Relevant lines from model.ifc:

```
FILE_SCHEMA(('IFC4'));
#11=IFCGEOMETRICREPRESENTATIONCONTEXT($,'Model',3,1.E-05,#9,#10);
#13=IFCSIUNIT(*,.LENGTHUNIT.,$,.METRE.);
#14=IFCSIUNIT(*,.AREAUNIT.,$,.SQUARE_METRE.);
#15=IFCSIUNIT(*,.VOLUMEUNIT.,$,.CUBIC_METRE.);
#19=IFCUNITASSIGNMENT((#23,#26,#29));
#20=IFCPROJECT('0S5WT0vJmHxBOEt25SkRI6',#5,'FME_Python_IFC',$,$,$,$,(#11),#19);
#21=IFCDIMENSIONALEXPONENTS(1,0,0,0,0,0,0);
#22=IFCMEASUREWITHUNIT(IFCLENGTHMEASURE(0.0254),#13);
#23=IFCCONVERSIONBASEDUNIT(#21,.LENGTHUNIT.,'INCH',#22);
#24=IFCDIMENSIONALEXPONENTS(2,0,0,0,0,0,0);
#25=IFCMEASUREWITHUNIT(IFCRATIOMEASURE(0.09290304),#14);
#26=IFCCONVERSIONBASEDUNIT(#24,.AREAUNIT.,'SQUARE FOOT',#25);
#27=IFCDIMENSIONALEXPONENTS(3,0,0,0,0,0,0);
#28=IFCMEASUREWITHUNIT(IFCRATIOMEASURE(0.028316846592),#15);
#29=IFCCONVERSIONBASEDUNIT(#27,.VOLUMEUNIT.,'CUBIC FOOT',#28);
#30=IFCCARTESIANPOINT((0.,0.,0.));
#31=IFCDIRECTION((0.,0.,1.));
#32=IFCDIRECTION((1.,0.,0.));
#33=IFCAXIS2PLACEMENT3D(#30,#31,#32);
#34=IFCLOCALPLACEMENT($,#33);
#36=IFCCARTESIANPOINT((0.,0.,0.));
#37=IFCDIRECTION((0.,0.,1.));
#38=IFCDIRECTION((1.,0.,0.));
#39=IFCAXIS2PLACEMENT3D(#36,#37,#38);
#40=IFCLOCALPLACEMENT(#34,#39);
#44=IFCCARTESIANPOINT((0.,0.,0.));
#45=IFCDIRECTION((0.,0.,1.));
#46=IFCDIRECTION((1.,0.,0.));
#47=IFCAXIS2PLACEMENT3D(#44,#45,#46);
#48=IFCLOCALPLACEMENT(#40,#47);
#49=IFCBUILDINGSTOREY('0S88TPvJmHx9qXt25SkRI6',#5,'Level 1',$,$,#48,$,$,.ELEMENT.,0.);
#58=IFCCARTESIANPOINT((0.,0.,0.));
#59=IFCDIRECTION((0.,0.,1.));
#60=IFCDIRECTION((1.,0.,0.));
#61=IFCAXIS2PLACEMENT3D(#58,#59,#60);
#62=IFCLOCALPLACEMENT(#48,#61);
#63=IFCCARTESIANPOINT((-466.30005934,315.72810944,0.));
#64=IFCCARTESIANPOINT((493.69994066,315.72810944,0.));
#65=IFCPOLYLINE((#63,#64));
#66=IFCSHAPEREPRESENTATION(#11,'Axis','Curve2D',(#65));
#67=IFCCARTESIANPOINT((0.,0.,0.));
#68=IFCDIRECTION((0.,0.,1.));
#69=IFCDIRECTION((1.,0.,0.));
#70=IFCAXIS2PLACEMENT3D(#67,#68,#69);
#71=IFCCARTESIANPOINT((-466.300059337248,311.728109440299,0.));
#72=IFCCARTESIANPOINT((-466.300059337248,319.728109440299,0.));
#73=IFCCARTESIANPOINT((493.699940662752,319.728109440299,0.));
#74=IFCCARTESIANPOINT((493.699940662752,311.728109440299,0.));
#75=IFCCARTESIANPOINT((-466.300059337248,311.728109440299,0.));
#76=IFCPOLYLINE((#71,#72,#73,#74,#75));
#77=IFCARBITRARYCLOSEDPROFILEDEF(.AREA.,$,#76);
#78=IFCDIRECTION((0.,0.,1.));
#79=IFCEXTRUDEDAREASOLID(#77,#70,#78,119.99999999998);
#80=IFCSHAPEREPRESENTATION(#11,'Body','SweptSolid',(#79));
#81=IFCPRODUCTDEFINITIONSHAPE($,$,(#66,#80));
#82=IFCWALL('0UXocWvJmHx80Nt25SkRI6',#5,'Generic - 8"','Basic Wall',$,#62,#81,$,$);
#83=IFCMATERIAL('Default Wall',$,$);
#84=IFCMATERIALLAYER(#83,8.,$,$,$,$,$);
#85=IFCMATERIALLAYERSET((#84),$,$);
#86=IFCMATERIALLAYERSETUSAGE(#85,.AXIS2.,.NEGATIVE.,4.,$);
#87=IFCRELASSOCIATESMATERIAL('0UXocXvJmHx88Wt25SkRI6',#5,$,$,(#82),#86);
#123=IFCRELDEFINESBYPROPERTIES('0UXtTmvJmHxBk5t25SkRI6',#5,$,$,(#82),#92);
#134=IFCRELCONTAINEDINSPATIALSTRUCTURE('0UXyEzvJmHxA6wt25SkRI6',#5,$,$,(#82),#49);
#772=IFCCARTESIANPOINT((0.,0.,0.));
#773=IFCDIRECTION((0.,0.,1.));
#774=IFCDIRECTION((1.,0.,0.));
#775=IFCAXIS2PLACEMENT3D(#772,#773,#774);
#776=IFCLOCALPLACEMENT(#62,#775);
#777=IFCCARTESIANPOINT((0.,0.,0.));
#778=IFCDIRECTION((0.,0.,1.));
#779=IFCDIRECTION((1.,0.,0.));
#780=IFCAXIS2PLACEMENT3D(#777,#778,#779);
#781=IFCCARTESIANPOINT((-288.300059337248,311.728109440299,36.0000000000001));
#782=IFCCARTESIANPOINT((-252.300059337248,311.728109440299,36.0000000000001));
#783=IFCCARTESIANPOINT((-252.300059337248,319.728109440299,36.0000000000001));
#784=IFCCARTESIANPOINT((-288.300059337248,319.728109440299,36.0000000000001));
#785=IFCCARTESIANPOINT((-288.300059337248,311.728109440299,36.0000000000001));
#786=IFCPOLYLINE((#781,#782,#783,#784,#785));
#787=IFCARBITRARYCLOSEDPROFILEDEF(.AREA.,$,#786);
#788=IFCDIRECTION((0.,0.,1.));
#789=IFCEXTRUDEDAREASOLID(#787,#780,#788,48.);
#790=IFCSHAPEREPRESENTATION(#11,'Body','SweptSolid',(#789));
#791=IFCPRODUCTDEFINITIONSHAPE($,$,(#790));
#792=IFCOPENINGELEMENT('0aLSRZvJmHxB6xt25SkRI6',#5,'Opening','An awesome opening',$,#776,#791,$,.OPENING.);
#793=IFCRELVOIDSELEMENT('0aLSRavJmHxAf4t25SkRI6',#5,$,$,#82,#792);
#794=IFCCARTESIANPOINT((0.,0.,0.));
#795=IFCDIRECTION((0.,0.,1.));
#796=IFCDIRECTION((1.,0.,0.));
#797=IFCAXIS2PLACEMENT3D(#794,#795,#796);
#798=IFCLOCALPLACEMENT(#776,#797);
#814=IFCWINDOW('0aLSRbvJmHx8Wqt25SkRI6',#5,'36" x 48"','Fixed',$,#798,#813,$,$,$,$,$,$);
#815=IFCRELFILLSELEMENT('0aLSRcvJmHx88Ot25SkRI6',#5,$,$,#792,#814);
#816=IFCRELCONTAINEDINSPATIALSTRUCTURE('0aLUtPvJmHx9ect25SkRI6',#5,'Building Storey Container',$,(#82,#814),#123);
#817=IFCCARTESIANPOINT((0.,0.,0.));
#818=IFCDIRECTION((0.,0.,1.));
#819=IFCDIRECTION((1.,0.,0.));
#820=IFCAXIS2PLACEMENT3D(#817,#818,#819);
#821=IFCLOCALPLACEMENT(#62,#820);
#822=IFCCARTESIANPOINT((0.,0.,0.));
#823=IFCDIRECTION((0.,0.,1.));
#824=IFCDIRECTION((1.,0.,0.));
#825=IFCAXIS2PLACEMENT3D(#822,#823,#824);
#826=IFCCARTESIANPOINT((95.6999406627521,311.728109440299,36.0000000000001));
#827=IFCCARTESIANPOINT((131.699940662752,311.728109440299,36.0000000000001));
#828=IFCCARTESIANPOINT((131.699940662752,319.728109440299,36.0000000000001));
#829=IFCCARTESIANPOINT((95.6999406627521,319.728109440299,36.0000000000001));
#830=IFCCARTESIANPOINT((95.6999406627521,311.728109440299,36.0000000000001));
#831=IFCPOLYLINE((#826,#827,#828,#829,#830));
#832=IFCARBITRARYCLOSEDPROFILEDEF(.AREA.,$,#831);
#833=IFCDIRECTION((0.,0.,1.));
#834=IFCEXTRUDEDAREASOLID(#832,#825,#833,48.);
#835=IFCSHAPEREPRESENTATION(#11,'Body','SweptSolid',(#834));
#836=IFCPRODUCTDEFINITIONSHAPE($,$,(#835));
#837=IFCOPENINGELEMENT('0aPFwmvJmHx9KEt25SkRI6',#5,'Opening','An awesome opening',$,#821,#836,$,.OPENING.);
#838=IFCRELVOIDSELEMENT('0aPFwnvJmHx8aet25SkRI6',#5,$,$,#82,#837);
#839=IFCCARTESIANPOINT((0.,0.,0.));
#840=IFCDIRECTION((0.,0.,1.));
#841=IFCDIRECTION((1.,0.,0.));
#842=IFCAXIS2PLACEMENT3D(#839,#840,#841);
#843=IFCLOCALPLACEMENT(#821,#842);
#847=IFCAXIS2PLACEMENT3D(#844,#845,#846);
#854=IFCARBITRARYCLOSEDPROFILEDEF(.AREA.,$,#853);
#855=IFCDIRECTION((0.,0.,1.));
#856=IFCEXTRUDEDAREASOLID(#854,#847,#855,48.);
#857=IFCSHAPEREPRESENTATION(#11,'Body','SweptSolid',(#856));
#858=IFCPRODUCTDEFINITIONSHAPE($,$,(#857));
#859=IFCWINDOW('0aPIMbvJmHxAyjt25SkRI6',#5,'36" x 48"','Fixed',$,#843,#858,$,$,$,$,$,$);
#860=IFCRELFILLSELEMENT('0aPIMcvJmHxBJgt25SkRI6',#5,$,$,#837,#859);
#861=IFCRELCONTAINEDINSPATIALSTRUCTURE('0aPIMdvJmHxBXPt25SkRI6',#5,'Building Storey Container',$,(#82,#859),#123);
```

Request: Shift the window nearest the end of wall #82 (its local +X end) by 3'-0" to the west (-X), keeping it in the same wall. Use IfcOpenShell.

```python
import ifcopenshell
import ifcopenshell.api.geometry
import ifcopenshell.util.placement
import ifcopenshell.util.unit

model = ifcopenshell.open("model.ifc")
unit_scale = ifcopenshell.util.unit.calculate_unit_scale(model)

window = model.by_id(859)
opening = window.FillsVoids[0].RelatingOpeningElement
wall = opening.VoidsElements[0].RelatingBuildingElement

wall_matrix = ifcopenshell.util.placement.get_local_placement(wall.ObjectPlacement)
shift = wall_matrix[:3, 0] * -36 * 0.0254 / unit_scale
before = ifcopenshell.util.placement.get_local_placement(window.ObjectPlacement)[:3, 3].copy()

# The window is placed relative to its opening, so it follows when the opening moves.
matrix = ifcopenshell.util.placement.get_local_placement(opening.ObjectPlacement)
matrix[:3, 3] += shift
ifcopenshell.api.geometry.edit_object_placement(
    model, product=opening, matrix=matrix, is_si=False, should_transform_children=True
)

after = ifcopenshell.util.placement.get_local_placement(window.ObjectPlacement)[:3, 3]
print("window moved by", (after - before).round(3) + 0.0)

model.write("model_updated.ifc")
```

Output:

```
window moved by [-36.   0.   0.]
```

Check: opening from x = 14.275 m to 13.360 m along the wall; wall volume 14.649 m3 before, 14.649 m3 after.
